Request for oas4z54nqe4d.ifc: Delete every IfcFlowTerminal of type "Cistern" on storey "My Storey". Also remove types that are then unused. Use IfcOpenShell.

First a look at what the model holds.

```python
import ifcopenshell
import ifcopenshell.util.element

model = ifcopenshell.open("oas4z54nqe4d.ifc")
print(model.schema)
storey = next(s for s in model.by_type("IfcBuildingStorey") if s.Name == "My Storey")
terminals = [e for e in ifcopenshell.util.element.get_decomposition(storey) if e.is_a("IfcFlowTerminal")]
seen = {}
for e in terminals:
    element_type = ifcopenshell.util.element.get_type(e)
    name = element_type.Name if element_type not in (None, e) else None
    seen[name] = seen.get(name, 0) + 1
for name, count in sorted(seen.items(), key=str):
    print(count, "x", name)
```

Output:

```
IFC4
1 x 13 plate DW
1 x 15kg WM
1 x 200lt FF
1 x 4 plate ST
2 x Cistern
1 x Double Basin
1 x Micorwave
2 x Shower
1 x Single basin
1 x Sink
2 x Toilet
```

```python
import ifcopenshell
import ifcopenshell.api.root
import ifcopenshell.util.element

model = ifcopenshell.open("oas4z54nqe4d.ifc")

storey = next(s for s in model.by_type("IfcBuildingStorey") if s.Name == "My Storey")
terminals = [e for e in ifcopenshell.util.element.get_decomposition(storey) if e.is_a("IfcFlowTerminal")]
targets = [e for e in terminals if (t := ifcopenshell.util.element.get_type(e)) not in (None, e) and t.Name == "Cistern"]
types = {ifcopenshell.util.element.get_type(e) for e in targets} - {None, *targets}

for e in targets:
    ifcopenshell.api.root.remove_product(model, product=e)
print(len(targets), "removed")

unused = [t for t in types if not ifcopenshell.util.element.get_types(t)]
for t in unused:
    ifcopenshell.api.root.remove_product(model, product=t)
print(len(unused), "unused types removed")

model.write("oas4z54nqe4d_edited.ifc")
```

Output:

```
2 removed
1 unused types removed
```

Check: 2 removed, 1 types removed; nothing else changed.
